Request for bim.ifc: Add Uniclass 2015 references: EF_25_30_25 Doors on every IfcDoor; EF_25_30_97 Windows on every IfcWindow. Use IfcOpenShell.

First a look at what the model holds.

```python
import ifcopenshell

model = ifcopenshell.open("bim.ifc")
print(model.schema)
print("classifications:", [c.Name for c in model.by_type("IfcClassification")])
for ifc_class in ("IfcDoor", "IfcRoof", "IfcStair", "IfcWall", "IfcWindow"):
    print(ifc_class, len(model.by_type(ifc_class)))
```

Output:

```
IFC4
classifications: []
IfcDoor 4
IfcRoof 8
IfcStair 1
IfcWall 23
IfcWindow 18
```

```python
import ifcopenshell
import ifcopenshell.api.classification

model = ifcopenshell.open("bim.ifc")

system = ifcopenshell.api.classification.add_classification(model, classification="Uniclass 2015")

codes = {
    "IfcDoor": ("EF_25_30_25", "Doors"),
    "IfcWindow": ("EF_25_30_97", "Windows"),
}
for ifc_class, (code, name) in codes.items():
    products = model.by_type(ifc_class)
    ifcopenshell.api.classification.add_reference(
        model, products=products, classification=system, identification=code, name=name
    )
    print(code, len(products))

model.write("bim-out.ifc")
```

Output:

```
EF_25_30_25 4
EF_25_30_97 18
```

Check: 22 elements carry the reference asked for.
